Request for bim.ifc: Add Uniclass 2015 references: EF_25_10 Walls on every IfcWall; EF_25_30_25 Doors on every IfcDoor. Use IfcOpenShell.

First a look at what the model holds.

```python
import ifcopenshell

model = ifcopenshell.open("bim.ifc")
print(model.schema)
print("classifications:", [c.Name for c in model.by_type("IfcClassification")])
for ifc_class in ("IfcDoor", "IfcRoof", "IfcStair", "IfcWall", "IfcWindow"):
    print(ifc_class, len(model.by_type(ifc_class)))
```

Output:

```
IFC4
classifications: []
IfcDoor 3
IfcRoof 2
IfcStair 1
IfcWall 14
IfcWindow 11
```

```python
import ifcopenshell
import ifcopenshell.api.classification

model = ifcopenshell.open("bim.ifc")

system = ifcopenshell.api.classification.add_classification(model, classification="Uniclass 2015")

codes = {
    "IfcWall": ("EF_25_10", "Walls"),
    "IfcDoor": ("EF_25_30_25", "Doors"),
}
for ifc_class, (code, name) in codes.items():
    products = model.by_type(ifc_class)
    ifcopenshell.api.classification.add_reference(
        model, products=products, classification=system, identification=code, name=name
    )
    print(code, len(products))

model.write("bim-out.ifc")
```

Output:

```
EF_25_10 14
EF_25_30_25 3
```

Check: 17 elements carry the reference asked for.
